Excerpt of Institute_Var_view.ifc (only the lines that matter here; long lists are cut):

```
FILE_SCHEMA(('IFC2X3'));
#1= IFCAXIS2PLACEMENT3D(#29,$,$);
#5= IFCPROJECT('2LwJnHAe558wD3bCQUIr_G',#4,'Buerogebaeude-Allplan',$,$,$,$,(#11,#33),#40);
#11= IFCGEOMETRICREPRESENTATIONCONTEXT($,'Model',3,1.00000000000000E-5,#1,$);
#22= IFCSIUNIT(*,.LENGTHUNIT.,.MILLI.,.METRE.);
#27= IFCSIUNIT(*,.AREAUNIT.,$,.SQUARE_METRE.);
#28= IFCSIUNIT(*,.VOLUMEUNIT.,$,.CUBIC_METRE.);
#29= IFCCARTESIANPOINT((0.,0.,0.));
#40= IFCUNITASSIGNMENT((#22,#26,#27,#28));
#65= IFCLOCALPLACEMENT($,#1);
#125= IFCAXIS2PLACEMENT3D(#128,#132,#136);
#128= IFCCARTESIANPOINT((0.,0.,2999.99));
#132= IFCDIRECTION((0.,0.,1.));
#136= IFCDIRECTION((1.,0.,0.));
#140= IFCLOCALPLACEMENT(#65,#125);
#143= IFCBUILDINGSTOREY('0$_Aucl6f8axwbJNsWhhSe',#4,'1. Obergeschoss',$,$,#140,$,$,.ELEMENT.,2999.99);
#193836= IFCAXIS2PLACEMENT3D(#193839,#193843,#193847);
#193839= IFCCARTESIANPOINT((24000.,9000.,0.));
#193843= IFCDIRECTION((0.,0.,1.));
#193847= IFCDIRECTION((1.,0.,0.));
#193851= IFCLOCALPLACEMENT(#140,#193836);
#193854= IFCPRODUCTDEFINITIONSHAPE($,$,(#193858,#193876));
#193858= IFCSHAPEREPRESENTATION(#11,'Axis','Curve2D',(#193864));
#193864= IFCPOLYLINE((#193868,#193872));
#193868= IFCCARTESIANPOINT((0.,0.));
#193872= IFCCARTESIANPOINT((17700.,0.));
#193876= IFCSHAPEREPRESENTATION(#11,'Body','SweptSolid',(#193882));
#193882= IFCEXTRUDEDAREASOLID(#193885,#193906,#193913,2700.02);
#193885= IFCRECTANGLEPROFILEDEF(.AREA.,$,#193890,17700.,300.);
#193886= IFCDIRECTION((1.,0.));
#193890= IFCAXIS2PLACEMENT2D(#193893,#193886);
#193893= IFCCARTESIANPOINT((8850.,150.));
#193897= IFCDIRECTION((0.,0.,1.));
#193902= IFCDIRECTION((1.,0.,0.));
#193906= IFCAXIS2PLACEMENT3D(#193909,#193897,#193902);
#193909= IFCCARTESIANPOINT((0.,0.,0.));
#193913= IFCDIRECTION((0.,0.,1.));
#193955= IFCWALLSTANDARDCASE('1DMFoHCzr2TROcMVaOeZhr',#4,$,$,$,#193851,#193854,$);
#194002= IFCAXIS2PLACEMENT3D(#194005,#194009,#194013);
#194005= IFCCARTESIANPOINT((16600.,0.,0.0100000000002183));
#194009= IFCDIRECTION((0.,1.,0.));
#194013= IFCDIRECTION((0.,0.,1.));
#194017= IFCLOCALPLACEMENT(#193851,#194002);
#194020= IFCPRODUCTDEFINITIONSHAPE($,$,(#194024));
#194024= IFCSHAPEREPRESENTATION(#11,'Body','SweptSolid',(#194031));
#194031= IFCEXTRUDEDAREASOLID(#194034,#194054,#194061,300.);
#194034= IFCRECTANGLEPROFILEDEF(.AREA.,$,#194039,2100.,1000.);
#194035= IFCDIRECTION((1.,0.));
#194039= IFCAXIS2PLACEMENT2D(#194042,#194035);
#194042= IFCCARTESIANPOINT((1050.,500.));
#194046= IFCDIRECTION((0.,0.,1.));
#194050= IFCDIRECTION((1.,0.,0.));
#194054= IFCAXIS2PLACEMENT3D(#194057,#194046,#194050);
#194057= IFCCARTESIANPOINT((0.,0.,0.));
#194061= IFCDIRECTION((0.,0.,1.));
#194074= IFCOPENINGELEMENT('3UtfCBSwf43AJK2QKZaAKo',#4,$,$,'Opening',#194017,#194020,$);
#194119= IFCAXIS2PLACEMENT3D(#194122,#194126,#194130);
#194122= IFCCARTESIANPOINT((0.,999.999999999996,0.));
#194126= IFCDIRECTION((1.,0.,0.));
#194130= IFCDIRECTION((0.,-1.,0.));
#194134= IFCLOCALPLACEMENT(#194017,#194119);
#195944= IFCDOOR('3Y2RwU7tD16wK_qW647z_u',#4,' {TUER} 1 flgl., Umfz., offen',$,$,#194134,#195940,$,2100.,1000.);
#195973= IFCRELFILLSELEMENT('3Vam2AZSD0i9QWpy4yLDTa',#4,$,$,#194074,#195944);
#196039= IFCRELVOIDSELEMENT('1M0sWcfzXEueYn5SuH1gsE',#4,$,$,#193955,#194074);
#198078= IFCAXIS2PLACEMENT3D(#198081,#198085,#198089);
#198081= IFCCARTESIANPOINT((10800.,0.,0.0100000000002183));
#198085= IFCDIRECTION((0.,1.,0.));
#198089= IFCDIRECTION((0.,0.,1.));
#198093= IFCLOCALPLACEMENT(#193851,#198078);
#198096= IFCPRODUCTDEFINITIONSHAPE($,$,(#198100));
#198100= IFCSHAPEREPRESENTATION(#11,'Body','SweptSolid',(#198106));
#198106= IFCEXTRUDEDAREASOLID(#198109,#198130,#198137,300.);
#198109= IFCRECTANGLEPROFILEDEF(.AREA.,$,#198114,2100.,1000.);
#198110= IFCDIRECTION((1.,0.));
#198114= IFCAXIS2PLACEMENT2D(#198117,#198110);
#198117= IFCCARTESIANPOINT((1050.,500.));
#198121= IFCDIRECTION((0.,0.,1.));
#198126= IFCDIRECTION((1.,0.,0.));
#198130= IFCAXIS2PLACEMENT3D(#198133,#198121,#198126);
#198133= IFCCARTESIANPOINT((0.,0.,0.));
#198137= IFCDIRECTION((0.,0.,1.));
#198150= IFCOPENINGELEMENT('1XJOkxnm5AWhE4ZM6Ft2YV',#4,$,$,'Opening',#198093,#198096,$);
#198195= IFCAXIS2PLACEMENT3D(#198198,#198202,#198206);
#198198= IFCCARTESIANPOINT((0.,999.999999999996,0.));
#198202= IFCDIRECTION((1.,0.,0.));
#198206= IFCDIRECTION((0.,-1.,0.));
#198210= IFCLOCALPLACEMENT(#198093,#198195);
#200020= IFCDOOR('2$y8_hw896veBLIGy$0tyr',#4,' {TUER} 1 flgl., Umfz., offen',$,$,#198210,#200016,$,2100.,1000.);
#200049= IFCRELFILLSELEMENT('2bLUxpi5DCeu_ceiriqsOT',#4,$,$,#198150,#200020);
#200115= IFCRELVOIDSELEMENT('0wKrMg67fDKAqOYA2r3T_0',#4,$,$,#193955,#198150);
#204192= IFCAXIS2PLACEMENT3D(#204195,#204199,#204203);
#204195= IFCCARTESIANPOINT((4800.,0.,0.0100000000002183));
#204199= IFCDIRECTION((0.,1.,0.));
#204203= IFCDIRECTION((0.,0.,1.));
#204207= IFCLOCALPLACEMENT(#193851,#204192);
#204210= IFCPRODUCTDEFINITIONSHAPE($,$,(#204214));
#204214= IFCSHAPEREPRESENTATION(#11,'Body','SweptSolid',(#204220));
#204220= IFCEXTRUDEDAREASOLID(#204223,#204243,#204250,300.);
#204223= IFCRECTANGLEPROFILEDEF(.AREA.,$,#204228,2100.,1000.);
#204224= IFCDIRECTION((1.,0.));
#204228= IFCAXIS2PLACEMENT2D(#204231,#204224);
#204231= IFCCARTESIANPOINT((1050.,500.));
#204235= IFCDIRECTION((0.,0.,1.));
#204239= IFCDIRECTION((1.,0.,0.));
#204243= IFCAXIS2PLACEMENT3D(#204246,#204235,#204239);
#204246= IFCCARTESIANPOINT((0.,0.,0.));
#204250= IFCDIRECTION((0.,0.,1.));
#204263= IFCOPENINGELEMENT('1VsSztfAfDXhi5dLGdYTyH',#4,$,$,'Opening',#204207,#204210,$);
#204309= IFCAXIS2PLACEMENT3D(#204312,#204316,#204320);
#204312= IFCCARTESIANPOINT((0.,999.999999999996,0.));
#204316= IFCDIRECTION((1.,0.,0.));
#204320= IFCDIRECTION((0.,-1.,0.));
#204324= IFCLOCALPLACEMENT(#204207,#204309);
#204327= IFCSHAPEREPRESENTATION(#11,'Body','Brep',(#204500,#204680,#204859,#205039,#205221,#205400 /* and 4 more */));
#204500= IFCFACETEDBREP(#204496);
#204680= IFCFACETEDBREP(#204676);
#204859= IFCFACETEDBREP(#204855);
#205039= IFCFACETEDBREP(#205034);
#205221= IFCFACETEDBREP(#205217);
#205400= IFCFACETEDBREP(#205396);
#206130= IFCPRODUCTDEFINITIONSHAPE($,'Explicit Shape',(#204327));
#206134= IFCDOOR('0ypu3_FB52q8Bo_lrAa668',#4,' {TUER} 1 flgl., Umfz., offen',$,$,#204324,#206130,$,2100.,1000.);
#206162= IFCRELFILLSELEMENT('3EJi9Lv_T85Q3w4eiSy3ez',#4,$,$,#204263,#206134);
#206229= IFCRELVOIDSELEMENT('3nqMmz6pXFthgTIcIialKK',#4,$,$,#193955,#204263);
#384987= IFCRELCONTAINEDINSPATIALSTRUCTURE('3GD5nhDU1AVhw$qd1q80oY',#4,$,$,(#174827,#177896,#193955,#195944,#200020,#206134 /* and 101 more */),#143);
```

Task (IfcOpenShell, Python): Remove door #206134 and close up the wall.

```python
import ifcopenshell
import ifcopenshell.api.feature
import ifcopenshell.api.root
import ifcopenshell.geom
import ifcopenshell.util.shape

model = ifcopenshell.open("Institute_Var_view.ifc")
settings = ifcopenshell.geom.settings()


def volume(element):
    """Net volume in cubic metres, openings subtracted."""
    shape = ifcopenshell.geom.create_shape(settings, element)
    return ifcopenshell.util.shape.get_volume(shape.geometry)


door = model.by_guid("0ypu3_FB52q8Bo_lrAa668")
opening = door.FillsVoids[0].RelatingOpeningElement
wall = opening.VoidsElements[0].RelatingBuildingElement
before = volume(wall)

ifcopenshell.api.root.remove_product(model, product=door)
ifcopenshell.api.feature.remove_feature(model, feature=opening)

after = volume(wall)

print(f"wall volume {before:.3f} -> {after:.3f} m3")

model.write("Institute_Var_view_edited.ifc")
```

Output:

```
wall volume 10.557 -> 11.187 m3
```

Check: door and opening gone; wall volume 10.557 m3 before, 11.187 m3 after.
